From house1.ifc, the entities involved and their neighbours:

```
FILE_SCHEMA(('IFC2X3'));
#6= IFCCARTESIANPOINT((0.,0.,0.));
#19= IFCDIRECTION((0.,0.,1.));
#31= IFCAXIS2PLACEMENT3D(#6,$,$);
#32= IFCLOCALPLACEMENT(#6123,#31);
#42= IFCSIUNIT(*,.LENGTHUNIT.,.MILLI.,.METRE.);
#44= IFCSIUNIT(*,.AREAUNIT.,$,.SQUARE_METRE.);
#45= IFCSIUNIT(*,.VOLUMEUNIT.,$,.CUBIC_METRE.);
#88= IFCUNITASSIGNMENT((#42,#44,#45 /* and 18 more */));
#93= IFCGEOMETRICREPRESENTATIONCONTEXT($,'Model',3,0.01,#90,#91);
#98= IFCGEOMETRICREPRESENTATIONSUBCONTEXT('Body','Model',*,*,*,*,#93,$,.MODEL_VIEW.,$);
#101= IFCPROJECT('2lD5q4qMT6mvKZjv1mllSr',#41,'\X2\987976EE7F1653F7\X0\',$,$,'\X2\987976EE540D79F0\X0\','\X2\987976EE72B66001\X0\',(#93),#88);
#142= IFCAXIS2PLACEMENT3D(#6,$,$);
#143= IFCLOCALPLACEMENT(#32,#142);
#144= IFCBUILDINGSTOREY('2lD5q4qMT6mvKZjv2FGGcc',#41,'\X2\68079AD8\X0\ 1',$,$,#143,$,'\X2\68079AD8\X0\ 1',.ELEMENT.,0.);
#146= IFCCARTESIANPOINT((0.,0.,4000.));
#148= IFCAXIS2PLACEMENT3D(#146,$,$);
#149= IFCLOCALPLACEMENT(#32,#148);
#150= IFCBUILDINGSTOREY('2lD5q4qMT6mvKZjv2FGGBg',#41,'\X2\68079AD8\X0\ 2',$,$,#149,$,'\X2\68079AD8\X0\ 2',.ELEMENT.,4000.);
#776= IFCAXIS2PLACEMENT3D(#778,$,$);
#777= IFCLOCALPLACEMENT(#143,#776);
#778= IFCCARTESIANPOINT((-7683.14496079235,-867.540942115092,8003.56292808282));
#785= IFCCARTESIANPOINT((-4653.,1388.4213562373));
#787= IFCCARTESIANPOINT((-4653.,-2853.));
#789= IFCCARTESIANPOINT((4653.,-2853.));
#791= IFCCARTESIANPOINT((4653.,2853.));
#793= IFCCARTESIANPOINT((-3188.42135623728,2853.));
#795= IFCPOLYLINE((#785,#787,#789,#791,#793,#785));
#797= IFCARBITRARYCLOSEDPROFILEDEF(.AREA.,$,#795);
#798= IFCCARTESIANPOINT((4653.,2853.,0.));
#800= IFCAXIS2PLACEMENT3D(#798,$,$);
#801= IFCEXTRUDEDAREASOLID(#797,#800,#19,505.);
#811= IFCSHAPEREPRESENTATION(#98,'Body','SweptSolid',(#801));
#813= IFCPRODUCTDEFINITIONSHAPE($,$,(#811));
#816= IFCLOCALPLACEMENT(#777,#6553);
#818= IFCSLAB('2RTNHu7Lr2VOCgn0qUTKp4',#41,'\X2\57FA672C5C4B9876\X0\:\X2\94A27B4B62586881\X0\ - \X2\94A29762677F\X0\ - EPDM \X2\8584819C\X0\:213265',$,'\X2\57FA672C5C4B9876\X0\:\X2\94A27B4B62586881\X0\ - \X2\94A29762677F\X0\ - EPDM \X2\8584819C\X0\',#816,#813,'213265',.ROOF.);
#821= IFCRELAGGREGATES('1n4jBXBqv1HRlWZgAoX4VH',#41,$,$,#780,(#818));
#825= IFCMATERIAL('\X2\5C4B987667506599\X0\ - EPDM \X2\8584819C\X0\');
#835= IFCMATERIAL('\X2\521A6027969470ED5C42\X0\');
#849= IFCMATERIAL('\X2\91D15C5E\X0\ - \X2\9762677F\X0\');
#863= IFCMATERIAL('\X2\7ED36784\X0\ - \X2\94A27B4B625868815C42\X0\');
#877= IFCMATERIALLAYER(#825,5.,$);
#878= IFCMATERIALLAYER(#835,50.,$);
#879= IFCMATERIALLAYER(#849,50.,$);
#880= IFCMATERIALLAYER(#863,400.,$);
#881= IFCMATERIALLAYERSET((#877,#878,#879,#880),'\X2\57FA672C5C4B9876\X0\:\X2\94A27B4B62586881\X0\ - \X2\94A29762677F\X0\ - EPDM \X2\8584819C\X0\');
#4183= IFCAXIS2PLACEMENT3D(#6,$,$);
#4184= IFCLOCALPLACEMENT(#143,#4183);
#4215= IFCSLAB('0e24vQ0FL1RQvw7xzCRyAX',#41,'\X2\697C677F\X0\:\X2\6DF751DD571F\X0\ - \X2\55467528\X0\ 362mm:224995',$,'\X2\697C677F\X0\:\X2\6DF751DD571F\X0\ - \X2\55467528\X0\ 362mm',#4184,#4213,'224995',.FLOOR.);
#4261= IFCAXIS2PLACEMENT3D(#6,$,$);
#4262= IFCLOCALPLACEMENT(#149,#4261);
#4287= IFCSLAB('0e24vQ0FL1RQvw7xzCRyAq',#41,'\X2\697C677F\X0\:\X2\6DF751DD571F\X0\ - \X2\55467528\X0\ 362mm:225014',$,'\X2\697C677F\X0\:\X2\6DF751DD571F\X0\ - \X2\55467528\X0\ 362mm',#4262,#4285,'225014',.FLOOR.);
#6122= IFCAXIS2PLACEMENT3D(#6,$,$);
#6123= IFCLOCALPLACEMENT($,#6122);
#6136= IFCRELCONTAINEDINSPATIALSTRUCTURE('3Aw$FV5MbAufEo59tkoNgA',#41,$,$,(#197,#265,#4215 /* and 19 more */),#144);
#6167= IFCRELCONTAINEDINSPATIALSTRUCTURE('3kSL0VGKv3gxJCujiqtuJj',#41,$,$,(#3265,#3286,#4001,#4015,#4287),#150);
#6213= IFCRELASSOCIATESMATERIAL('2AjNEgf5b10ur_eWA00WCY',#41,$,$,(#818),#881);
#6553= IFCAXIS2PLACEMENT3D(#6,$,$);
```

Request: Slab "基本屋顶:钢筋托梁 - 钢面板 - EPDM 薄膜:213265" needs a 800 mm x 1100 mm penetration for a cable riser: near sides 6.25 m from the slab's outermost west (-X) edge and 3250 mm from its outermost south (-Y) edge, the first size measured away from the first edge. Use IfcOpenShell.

```python
import numpy as np
import ifcopenshell
import ifcopenshell.api.feature
import ifcopenshell.api.geometry
import ifcopenshell.api.root
import ifcopenshell.geom
import ifcopenshell.util.placement
import ifcopenshell.util.representation
import ifcopenshell.util.shape
import ifcopenshell.util.unit

model = ifcopenshell.open("house1.ifc")
unit_scale = ifcopenshell.util.unit.calculate_unit_scale(model)
settings = ifcopenshell.geom.settings()


def volume(element):
    """Net volume in cubic metres, openings subtracted."""
    shape = ifcopenshell.geom.create_shape(settings, element)
    return ifcopenshell.util.shape.get_volume(shape.geometry)


slab = model.by_guid("2RTNHu7Lr2VOCgn0qUTKp4")
before = volume(slab)

# Extent in the slab's own axes, in metres. The edges named are its -X and -Y sides.
slab_shape = ifcopenshell.geom.create_shape(settings, slab)
vertices = ifcopenshell.util.shape.get_vertices(slab_shape.geometry)
x_min, y_min, bottom = vertices.min(axis=0)
top = vertices[:, 2].max()

opening = ifcopenshell.api.root.create_entity(model, ifc_class="IfcOpeningElement", name="Cable riser opening")
context = ifcopenshell.util.representation.get_context(model, "Model", "Body", "MODEL_VIEW")
width, depth = 0.8, 1.1
outline = [(0.0, 0.0), (width, 0.0), (width, depth), (0.0, depth), (0.0, 0.0)]
# Overshoot both faces by 50 mm so the cut is clean.
shape = ifcopenshell.api.geometry.add_slab_representation(
    model, context=context, depth=top - bottom + 0.1, polyline=outline
)
ifcopenshell.api.geometry.assign_representation(model, product=opening, representation=shape)

matrix = ifcopenshell.util.placement.get_local_placement(slab.ObjectPlacement)
matrix[:, 3] = matrix @ np.append(np.array([x_min + 6.25, y_min + 3.25, bottom - 0.05]) / unit_scale, 1.0)
ifcopenshell.api.geometry.edit_object_placement(model, product=opening, matrix=matrix, is_si=False)
ifcopenshell.api.feature.add_feature(model, feature=opening, element=slab)

after = volume(slab)

print(f"slab volume {before:.3f} -> {after:.3f} m3")

model.write("house1_rev.ifc")
```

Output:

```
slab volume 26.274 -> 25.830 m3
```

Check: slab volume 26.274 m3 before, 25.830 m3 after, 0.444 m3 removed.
